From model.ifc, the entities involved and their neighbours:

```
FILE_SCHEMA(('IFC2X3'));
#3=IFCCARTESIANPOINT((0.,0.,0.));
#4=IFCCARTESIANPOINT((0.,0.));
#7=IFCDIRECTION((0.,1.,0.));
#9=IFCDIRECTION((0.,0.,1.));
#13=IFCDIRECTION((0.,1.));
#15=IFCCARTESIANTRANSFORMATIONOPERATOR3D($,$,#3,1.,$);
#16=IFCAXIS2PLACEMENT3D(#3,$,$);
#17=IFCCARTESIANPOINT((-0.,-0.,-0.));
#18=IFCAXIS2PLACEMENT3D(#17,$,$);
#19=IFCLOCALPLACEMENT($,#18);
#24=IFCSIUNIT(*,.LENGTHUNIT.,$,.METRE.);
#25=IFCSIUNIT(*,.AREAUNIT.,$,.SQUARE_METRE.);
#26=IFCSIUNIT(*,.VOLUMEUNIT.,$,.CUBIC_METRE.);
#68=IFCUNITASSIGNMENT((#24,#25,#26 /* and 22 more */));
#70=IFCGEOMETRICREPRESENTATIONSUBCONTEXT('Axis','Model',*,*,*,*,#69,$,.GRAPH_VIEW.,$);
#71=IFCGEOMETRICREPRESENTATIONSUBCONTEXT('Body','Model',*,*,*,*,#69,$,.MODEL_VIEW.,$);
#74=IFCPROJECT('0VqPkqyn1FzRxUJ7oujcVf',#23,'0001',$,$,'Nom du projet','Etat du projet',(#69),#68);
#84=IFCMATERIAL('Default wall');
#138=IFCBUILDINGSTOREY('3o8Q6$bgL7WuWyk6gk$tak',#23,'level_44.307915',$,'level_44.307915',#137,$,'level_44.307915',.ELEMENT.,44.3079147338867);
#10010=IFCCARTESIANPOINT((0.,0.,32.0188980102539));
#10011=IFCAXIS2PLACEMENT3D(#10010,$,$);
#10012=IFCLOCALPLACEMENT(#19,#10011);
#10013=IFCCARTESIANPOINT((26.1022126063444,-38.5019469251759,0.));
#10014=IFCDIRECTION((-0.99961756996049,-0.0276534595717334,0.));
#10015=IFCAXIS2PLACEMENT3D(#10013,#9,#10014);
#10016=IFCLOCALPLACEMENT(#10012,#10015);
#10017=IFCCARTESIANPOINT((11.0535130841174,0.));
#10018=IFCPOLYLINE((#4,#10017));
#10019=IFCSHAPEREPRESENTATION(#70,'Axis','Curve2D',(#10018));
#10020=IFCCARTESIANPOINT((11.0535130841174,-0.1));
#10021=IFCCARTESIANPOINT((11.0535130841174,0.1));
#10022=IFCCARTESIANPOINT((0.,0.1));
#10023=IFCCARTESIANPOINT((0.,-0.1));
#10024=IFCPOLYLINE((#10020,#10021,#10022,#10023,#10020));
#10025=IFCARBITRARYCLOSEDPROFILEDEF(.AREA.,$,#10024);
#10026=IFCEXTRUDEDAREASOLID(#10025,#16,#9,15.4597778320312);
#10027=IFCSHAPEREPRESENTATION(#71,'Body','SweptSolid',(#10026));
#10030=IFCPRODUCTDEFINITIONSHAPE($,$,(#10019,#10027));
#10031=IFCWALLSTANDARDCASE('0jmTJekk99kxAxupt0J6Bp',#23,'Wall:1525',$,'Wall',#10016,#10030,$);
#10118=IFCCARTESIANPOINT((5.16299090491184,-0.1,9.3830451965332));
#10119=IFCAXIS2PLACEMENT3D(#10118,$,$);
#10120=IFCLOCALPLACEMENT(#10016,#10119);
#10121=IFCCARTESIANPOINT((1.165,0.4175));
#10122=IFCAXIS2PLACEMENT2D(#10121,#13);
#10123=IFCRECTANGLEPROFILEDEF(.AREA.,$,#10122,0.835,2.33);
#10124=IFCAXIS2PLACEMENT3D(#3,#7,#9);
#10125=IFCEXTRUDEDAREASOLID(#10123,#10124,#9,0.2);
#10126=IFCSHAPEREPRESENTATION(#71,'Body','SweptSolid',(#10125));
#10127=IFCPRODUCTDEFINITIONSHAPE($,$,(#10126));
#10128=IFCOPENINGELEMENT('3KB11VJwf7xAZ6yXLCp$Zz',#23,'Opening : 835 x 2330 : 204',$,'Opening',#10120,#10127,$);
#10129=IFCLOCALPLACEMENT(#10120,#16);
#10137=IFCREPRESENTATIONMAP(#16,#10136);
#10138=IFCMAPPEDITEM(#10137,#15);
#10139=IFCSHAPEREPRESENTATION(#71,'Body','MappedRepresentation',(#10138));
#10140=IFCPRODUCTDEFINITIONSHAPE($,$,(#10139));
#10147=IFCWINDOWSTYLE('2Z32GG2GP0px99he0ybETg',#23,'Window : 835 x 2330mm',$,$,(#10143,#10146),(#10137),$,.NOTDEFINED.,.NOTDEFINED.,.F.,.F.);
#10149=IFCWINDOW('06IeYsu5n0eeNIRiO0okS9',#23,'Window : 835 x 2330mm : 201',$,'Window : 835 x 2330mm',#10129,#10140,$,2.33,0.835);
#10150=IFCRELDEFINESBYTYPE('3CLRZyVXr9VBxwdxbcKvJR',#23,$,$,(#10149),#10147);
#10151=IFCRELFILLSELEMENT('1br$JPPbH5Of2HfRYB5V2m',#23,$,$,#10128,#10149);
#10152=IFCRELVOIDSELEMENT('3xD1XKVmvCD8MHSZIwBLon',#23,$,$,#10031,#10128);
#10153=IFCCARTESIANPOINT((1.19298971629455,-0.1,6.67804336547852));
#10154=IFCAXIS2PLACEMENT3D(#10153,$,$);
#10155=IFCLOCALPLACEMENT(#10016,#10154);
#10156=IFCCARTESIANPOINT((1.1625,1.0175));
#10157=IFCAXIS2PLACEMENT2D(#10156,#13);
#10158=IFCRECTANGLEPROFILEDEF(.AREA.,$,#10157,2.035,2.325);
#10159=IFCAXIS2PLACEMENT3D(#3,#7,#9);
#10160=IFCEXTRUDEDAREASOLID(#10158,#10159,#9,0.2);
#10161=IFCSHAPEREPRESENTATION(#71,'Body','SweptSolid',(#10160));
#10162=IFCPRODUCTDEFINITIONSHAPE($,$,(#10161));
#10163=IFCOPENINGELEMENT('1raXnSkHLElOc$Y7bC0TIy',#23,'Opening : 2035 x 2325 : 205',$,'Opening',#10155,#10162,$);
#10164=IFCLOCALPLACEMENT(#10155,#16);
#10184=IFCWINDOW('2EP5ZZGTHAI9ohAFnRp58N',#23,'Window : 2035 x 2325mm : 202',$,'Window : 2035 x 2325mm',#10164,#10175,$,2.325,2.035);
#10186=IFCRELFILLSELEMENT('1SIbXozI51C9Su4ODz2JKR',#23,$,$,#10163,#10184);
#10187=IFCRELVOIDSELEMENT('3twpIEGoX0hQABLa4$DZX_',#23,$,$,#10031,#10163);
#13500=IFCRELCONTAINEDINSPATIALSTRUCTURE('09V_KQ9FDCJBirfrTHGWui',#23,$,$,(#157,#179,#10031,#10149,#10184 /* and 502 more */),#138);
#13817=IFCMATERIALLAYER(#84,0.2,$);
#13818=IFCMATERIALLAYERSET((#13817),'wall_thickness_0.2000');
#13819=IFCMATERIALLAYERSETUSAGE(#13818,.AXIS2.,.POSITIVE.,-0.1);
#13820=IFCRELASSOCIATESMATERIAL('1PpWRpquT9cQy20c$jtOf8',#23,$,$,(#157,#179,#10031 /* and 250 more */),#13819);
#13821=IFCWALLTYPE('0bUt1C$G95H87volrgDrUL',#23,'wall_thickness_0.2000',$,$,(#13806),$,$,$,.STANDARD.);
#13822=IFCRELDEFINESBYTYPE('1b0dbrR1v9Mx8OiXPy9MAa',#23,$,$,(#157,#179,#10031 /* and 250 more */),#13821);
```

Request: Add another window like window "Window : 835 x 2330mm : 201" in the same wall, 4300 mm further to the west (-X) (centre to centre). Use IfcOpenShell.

```python
import ifcopenshell
import ifcopenshell.api.feature
import ifcopenshell.api.geometry
import ifcopenshell.api.root
import ifcopenshell.geom
import ifcopenshell.util.element
import ifcopenshell.util.placement
import ifcopenshell.util.shape
import ifcopenshell.util.unit

model = ifcopenshell.open("model.ifc")
unit_scale = ifcopenshell.util.unit.calculate_unit_scale(model)
settings = ifcopenshell.geom.settings()


def volume(element):
    """Net volume in cubic metres, openings subtracted."""
    shape = ifcopenshell.geom.create_shape(settings, element)
    return ifcopenshell.util.shape.get_volume(shape.geometry)


window = model.by_guid("06IeYsu5n0eeNIRiO0okS9")
opening = window.FillsVoids[0].RelatingOpeningElement
wall = opening.VoidsElements[0].RelatingBuildingElement
before = volume(wall)
shift = ifcopenshell.util.placement.get_local_placement(wall.ObjectPlacement)[:3, 0] * 4.3 / unit_scale

# copy_class copies the void relationship, type, container and properties, but no geometry.
new_opening = ifcopenshell.api.root.copy_class(model, product=opening)
new_opening.Representation = ifcopenshell.util.element.copy_deep(
    model, opening.Representation, exclude=["IfcGeometricRepresentationContext", "IfcRepresentationMap"]
)
new_opening.Name = "Opening : 835 x 2330"
new_window = ifcopenshell.api.root.copy_class(model, product=window)
new_window.Representation = ifcopenshell.util.element.copy_deep(
    model, window.Representation, exclude=["IfcGeometricRepresentationContext", "IfcRepresentationMap"]
)
new_window.Name = "Window : 835 x 2330mm"
fills = ifcopenshell.api.feature.add_filling(model, opening=new_opening, element=new_window)
fills.OwnerHistory = new_window.OwnerHistory  # required in IFC2X3

for old, new in ((opening, new_opening), (window, new_window)):
    matrix = ifcopenshell.util.placement.get_local_placement(old.ObjectPlacement)
    matrix[:3, 3] += shift
    ifcopenshell.api.geometry.edit_object_placement(model, product=new, matrix=matrix, is_si=False)

after = volume(wall)

print(f"wall volume {before:.3f} -> {after:.3f} m3")

model.write("model_edited.ifc")
```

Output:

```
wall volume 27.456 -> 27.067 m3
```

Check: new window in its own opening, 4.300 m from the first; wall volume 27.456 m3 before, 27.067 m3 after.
